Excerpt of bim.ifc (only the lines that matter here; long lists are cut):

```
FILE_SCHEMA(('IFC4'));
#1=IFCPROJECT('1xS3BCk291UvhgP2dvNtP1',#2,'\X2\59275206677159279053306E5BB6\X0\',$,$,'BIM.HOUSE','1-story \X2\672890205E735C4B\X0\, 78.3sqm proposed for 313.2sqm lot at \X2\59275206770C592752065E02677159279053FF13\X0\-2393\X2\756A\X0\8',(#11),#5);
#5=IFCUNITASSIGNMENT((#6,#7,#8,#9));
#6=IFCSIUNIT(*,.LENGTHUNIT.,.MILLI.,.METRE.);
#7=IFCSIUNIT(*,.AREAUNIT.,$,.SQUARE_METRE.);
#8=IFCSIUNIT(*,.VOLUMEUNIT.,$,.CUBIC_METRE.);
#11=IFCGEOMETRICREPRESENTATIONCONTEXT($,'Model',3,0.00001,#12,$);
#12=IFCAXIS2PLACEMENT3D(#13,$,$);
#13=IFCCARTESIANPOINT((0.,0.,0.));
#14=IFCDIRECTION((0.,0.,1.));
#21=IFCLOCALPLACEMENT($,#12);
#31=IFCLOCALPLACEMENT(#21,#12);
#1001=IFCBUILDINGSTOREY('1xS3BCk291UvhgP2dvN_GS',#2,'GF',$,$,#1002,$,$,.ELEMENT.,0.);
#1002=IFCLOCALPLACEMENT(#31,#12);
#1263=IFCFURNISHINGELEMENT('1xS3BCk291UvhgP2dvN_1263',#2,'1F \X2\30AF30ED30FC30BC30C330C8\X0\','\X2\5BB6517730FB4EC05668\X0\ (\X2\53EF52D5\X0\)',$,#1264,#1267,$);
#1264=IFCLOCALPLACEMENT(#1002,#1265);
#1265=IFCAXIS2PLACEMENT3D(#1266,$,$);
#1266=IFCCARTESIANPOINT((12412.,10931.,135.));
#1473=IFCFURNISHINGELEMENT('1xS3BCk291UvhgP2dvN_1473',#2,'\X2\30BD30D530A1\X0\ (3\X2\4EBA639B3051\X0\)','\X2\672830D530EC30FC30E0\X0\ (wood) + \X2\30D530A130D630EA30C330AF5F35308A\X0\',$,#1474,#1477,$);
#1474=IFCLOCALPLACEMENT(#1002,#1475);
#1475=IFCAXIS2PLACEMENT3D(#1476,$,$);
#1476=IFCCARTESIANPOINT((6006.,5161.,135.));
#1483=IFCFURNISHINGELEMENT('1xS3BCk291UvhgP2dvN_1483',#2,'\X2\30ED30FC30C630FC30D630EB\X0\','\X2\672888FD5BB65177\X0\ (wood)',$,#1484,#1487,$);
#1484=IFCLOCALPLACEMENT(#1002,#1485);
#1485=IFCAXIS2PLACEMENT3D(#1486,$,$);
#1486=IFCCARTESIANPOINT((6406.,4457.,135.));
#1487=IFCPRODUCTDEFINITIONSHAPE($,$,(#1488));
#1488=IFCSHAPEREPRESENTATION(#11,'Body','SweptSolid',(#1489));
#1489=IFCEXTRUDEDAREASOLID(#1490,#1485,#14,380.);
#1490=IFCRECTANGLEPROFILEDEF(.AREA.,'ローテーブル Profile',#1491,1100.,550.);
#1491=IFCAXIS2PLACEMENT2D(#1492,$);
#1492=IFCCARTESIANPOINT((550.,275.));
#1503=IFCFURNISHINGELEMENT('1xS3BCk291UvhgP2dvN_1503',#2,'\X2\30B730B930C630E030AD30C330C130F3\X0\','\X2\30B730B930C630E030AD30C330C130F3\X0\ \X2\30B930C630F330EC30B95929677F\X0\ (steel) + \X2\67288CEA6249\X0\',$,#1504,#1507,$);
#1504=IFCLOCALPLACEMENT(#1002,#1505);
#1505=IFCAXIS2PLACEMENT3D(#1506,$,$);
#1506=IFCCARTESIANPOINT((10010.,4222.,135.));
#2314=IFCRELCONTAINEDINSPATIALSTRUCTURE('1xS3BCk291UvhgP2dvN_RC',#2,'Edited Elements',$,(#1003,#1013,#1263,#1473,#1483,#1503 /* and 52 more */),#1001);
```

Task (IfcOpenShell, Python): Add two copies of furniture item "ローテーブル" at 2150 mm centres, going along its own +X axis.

```python
import ifcopenshell
import ifcopenshell.api.geometry
import ifcopenshell.api.root
import ifcopenshell.util.element
import ifcopenshell.util.placement
import ifcopenshell.util.unit

model = ifcopenshell.open("bim.ifc")
unit_scale = ifcopenshell.util.unit.calculate_unit_scale(model)


def reuse_history(source, copy):
    """copy_class also copies each property set's owner history, people and application; keep the originals."""
    for rel in copy.IsDefinedBy:
        if rel.is_a("IfcRelDefinesByProperties") and (history := rel.RelatingPropertyDefinition.OwnerHistory):
            rel.RelatingPropertyDefinition.OwnerHistory = source.OwnerHistory
            ifcopenshell.util.element.remove_deep2(model, history)


source = model.by_guid("1xS3BCk291UvhgP2dvN_1483")
base = ifcopenshell.util.placement.get_local_placement(source.ObjectPlacement)
step = base[:3, 0] * 2.15 / unit_scale

for i in range(1, 3):
    copy = ifcopenshell.api.root.copy_class(model, product=source)
    copy.Representation = ifcopenshell.util.element.copy_deep(
        model, source.Representation, exclude=["IfcGeometricRepresentationContext", "IfcRepresentationMap"]
    )
    reuse_history(source, copy)
    matrix = base.copy()
    matrix[:3, 3] += i * step
    print("added at", matrix[:3, 3].round(3) + 0.0)
    ifcopenshell.api.geometry.edit_object_placement(model, product=copy, matrix=matrix, is_si=False)

model.write("bim_updated.ifc")
```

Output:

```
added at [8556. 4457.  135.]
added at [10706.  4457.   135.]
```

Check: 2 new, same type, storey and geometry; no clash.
